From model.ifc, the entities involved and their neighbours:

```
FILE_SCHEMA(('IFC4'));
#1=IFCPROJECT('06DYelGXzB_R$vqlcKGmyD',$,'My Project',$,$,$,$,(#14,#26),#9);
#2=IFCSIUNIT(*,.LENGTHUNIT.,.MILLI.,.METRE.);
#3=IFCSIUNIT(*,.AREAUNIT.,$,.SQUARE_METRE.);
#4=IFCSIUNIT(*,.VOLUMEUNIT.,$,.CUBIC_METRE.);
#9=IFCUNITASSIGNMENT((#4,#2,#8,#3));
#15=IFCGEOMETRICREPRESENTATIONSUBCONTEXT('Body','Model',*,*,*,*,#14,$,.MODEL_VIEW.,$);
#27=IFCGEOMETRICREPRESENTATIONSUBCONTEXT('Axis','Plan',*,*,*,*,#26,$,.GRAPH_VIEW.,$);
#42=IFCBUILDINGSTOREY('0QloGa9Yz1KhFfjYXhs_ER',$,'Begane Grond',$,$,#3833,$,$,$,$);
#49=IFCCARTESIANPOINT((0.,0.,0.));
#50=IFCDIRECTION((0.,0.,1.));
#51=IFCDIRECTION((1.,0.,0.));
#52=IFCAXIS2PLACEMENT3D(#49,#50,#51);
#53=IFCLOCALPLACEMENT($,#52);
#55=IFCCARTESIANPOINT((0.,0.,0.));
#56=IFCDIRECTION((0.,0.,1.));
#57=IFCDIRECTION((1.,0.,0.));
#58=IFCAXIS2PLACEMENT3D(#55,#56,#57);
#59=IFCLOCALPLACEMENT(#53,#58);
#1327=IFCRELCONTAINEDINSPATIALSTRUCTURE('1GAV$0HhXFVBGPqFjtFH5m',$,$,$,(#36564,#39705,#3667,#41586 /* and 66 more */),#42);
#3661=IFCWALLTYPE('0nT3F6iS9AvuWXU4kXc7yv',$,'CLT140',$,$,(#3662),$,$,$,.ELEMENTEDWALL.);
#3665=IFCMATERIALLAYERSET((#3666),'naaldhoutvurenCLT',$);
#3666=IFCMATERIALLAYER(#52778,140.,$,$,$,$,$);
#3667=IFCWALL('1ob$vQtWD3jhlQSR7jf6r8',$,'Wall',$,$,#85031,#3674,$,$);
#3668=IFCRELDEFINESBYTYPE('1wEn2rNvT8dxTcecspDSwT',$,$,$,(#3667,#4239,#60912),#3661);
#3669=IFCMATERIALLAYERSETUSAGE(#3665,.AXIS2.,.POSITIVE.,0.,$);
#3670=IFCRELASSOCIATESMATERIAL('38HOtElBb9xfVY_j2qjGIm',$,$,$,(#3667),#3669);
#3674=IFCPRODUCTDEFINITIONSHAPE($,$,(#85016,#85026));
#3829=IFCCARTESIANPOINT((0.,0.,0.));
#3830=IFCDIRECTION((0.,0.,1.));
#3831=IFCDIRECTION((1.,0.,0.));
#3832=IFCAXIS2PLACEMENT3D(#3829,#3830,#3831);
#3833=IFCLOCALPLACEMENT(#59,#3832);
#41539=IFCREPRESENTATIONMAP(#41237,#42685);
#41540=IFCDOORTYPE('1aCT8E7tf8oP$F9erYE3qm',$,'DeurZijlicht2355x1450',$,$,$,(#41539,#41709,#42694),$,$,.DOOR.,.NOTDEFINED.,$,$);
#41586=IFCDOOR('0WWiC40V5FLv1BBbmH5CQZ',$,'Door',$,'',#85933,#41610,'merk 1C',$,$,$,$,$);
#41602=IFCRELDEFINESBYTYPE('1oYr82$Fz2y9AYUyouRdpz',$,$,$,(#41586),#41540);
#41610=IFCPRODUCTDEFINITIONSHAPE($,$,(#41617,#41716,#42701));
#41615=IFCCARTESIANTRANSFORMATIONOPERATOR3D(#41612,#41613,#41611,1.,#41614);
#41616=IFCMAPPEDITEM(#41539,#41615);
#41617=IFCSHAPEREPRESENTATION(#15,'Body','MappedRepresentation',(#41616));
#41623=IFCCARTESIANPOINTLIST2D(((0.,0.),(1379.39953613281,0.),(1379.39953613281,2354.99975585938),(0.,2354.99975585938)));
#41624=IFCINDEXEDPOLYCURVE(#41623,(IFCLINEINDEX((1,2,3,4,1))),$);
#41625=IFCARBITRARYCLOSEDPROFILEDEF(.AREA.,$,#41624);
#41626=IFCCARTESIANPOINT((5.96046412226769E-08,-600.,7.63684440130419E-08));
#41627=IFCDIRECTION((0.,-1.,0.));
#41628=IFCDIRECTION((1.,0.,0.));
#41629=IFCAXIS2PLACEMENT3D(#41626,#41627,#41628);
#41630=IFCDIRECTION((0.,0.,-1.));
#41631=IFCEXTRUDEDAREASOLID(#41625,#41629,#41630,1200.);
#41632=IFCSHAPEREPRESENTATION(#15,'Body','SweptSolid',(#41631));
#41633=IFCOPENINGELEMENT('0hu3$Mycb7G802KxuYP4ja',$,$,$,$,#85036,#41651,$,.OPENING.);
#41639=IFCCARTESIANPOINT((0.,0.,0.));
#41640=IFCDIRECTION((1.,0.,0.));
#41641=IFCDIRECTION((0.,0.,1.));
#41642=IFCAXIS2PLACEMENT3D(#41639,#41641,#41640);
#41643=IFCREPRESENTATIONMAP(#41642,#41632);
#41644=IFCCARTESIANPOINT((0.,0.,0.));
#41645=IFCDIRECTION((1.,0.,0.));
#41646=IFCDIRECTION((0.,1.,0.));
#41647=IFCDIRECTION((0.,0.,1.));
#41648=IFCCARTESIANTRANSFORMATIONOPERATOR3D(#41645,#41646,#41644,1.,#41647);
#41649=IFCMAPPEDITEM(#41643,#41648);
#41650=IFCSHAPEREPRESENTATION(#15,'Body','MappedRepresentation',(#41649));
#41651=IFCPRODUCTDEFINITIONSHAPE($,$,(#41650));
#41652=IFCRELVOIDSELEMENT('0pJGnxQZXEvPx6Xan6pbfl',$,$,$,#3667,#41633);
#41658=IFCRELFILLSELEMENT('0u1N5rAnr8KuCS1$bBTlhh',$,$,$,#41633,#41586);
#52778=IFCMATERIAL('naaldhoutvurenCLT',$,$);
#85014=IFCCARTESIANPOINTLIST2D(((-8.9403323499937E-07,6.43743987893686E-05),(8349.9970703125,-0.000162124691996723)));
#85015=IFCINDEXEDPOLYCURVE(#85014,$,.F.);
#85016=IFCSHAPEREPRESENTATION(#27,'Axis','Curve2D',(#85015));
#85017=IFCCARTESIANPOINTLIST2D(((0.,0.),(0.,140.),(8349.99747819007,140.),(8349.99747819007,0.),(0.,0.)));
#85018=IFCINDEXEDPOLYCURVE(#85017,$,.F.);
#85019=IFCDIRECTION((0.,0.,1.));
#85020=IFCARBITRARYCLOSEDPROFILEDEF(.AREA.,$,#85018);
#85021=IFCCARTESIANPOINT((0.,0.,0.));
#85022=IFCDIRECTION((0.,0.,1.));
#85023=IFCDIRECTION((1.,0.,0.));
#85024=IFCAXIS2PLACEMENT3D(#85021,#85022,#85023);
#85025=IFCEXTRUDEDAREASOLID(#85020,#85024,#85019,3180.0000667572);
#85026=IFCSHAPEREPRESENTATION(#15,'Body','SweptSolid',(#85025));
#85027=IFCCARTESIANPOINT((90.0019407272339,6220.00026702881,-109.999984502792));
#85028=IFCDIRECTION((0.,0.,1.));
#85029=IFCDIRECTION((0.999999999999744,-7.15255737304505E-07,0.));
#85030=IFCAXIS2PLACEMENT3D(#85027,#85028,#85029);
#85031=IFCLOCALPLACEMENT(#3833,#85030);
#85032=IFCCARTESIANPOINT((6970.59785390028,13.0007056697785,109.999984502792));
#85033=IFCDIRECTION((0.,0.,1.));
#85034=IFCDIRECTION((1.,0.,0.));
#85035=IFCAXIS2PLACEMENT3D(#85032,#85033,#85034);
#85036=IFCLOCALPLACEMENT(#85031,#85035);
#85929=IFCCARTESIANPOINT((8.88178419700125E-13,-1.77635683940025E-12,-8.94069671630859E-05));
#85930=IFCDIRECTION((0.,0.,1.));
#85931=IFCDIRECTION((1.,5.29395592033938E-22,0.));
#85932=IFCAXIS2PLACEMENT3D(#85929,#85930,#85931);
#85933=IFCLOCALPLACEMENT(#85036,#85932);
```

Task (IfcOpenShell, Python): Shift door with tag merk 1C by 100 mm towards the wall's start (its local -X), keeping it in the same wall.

```python
import ifcopenshell
import ifcopenshell.api.geometry
import ifcopenshell.util.placement

model = ifcopenshell.open("model.ifc")

door = model.by_guid("0WWiC40V5FLv1BBbmH5CQZ")
opening = door.FillsVoids[0].RelatingOpeningElement
wall = opening.VoidsElements[0].RelatingBuildingElement

wall_matrix = ifcopenshell.util.placement.get_local_placement(wall.ObjectPlacement)
shift = wall_matrix[:3, 0] * -100.0
before = ifcopenshell.util.placement.get_local_placement(door.ObjectPlacement)[:3, 3].copy()

# The door is placed relative to its opening, so it follows when the opening moves.
matrix = ifcopenshell.util.placement.get_local_placement(opening.ObjectPlacement)
matrix[:3, 3] += shift
ifcopenshell.api.geometry.edit_object_placement(
    model, product=opening, matrix=matrix, is_si=False, should_transform_children=True
)

after = ifcopenshell.util.placement.get_local_placement(door.ObjectPlacement)[:3, 3]
print("door moved by", (after - before).round(3) + 0.0)

model.write("model_rev.ifc")
```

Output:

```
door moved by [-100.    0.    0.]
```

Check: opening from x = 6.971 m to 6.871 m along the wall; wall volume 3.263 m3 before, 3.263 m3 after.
